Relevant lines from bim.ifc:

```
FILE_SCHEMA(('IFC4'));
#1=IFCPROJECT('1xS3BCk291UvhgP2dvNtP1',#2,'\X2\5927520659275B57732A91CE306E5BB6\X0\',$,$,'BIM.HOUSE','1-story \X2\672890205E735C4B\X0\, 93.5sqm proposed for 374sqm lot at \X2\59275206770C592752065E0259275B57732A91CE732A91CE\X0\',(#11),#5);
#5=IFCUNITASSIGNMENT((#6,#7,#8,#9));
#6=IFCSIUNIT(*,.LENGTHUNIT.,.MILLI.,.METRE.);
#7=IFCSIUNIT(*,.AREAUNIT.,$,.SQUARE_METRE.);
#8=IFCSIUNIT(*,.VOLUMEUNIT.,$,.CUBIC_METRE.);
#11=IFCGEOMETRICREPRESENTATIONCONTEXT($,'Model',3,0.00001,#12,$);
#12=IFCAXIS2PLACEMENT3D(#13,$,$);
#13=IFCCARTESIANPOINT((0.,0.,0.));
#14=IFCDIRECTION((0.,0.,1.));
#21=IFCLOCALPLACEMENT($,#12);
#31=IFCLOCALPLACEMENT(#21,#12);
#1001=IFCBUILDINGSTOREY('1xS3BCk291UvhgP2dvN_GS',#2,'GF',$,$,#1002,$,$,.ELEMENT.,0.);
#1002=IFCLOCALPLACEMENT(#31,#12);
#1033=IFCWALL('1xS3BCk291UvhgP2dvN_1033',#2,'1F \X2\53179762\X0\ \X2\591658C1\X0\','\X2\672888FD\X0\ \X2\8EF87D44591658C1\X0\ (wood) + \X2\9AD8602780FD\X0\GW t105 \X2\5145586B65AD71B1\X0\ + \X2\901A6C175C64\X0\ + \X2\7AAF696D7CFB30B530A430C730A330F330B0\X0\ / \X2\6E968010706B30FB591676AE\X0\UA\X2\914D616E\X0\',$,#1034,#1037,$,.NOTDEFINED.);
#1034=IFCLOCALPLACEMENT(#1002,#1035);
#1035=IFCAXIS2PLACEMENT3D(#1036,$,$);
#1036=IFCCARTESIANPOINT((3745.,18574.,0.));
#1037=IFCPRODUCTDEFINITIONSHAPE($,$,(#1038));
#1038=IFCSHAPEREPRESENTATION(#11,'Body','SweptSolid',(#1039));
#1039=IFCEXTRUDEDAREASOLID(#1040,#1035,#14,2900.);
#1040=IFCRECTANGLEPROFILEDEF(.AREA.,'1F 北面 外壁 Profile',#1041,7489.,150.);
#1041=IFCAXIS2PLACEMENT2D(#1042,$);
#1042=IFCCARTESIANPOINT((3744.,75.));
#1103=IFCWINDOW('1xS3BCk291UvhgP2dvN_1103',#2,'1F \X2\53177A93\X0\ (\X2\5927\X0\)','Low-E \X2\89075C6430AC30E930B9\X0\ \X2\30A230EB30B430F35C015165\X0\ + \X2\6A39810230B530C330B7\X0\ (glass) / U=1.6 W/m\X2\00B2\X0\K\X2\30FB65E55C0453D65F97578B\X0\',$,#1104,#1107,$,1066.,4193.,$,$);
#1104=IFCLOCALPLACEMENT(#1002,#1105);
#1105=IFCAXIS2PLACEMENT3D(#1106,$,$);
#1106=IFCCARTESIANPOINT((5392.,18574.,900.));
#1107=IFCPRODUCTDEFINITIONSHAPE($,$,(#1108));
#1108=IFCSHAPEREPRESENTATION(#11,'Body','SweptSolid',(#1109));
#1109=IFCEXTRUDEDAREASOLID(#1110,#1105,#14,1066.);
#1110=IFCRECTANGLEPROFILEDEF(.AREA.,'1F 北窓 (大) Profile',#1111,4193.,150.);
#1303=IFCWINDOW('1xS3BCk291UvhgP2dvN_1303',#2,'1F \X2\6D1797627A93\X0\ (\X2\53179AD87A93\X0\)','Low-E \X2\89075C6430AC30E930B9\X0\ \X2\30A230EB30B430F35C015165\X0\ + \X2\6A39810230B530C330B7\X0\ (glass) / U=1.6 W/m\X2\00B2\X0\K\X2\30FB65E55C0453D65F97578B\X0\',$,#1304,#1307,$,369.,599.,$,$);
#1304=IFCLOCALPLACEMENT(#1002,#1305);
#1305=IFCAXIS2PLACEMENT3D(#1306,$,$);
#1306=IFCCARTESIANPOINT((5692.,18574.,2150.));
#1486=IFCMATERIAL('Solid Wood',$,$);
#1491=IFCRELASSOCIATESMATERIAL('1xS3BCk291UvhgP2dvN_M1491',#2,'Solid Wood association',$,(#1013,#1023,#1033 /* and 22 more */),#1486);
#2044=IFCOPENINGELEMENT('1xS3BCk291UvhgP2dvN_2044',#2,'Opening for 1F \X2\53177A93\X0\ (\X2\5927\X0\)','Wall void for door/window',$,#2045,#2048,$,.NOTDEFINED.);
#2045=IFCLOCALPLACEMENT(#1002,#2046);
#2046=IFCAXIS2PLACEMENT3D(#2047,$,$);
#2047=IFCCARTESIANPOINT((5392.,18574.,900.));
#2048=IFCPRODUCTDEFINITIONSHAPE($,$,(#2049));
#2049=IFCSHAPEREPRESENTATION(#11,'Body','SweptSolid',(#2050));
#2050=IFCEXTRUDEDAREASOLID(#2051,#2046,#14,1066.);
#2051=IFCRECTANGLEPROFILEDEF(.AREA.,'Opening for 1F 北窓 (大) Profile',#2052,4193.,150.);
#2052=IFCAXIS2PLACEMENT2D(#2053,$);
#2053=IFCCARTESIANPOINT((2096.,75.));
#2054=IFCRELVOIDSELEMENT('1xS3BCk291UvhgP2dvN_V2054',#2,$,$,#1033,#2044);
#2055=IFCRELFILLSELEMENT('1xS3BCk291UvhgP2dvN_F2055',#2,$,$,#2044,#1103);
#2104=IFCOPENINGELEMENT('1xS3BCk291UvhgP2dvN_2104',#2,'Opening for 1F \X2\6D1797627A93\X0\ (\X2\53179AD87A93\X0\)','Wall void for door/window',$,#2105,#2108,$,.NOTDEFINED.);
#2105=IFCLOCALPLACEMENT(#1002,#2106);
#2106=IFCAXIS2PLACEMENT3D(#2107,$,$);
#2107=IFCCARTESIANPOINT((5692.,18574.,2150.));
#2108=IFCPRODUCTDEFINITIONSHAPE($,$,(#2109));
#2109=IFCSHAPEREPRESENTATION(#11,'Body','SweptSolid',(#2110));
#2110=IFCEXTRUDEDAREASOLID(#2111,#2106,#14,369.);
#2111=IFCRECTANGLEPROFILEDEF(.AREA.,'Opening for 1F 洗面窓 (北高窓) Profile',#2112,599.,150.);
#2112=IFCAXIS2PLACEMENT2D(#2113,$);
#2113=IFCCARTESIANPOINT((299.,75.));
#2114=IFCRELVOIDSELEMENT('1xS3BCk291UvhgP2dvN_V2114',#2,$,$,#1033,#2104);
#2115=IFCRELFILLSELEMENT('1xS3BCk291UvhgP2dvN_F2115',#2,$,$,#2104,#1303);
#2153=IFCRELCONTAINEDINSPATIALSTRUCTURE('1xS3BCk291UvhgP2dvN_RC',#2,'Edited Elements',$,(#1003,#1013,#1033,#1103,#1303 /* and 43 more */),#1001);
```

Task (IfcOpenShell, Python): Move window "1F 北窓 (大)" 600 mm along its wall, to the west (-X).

```python
import ifcopenshell
import ifcopenshell.api.geometry
import ifcopenshell.util.placement
import ifcopenshell.util.unit

model = ifcopenshell.open("bim.ifc")
unit_scale = ifcopenshell.util.unit.calculate_unit_scale(model)

window = model.by_id(1103)
opening = window.FillsVoids[0].RelatingOpeningElement
wall = opening.VoidsElements[0].RelatingBuildingElement

wall_matrix = ifcopenshell.util.placement.get_local_placement(wall.ObjectPlacement)
shift = wall_matrix[:3, 0] * -0.6 / unit_scale
before = ifcopenshell.util.placement.get_local_placement(window.ObjectPlacement)[:3, 3].copy()

# The window is not placed relative to its opening, so move both.
for product in (opening, window):
    matrix = ifcopenshell.util.placement.get_local_placement(product.ObjectPlacement)
    matrix[:3, 3] += shift
    ifcopenshell.api.geometry.edit_object_placement(model, product=product, matrix=matrix, is_si=False)

after = ifcopenshell.util.placement.get_local_placement(window.ObjectPlacement)[:3, 3]
print("window moved by", (after - before).round(3) + 0.0)

model.write("bim_edited.ifc")
```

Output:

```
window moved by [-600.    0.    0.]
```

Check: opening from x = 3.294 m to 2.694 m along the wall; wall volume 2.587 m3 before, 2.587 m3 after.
